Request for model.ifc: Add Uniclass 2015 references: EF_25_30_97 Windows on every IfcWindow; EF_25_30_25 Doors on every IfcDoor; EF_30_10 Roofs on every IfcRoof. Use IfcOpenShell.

First a look at what the model holds.

```python
import ifcopenshell

model = ifcopenshell.open("model.ifc")
print(model.schema)
print("classifications:", [c.Name for c in model.by_type("IfcClassification")])
for ifc_class in ("IfcDoor", "IfcRoof", "IfcStair", "IfcWall", "IfcWindow"):
    print(ifc_class, len(model.by_type(ifc_class)))
```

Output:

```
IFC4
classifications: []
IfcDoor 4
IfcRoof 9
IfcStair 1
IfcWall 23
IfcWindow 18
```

```python
import ifcopenshell
import ifcopenshell.api.classification

model = ifcopenshell.open("model.ifc")

system = ifcopenshell.api.classification.add_classification(model, classification="Uniclass 2015")

codes = {
    "IfcWindow": ("EF_25_30_97", "Windows"),
    "IfcDoor": ("EF_25_30_25", "Doors"),
    "IfcRoof": ("EF_30_10", "Roofs"),
}
for ifc_class, (code, name) in codes.items():
    products = model.by_type(ifc_class)
    ifcopenshell.api.classification.add_reference(
        model, products=products, classification=system, identification=code, name=name
    )
    print(code, len(products))

model.write("model_v2.ifc")
```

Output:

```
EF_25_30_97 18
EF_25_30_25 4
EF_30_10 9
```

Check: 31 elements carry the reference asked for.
